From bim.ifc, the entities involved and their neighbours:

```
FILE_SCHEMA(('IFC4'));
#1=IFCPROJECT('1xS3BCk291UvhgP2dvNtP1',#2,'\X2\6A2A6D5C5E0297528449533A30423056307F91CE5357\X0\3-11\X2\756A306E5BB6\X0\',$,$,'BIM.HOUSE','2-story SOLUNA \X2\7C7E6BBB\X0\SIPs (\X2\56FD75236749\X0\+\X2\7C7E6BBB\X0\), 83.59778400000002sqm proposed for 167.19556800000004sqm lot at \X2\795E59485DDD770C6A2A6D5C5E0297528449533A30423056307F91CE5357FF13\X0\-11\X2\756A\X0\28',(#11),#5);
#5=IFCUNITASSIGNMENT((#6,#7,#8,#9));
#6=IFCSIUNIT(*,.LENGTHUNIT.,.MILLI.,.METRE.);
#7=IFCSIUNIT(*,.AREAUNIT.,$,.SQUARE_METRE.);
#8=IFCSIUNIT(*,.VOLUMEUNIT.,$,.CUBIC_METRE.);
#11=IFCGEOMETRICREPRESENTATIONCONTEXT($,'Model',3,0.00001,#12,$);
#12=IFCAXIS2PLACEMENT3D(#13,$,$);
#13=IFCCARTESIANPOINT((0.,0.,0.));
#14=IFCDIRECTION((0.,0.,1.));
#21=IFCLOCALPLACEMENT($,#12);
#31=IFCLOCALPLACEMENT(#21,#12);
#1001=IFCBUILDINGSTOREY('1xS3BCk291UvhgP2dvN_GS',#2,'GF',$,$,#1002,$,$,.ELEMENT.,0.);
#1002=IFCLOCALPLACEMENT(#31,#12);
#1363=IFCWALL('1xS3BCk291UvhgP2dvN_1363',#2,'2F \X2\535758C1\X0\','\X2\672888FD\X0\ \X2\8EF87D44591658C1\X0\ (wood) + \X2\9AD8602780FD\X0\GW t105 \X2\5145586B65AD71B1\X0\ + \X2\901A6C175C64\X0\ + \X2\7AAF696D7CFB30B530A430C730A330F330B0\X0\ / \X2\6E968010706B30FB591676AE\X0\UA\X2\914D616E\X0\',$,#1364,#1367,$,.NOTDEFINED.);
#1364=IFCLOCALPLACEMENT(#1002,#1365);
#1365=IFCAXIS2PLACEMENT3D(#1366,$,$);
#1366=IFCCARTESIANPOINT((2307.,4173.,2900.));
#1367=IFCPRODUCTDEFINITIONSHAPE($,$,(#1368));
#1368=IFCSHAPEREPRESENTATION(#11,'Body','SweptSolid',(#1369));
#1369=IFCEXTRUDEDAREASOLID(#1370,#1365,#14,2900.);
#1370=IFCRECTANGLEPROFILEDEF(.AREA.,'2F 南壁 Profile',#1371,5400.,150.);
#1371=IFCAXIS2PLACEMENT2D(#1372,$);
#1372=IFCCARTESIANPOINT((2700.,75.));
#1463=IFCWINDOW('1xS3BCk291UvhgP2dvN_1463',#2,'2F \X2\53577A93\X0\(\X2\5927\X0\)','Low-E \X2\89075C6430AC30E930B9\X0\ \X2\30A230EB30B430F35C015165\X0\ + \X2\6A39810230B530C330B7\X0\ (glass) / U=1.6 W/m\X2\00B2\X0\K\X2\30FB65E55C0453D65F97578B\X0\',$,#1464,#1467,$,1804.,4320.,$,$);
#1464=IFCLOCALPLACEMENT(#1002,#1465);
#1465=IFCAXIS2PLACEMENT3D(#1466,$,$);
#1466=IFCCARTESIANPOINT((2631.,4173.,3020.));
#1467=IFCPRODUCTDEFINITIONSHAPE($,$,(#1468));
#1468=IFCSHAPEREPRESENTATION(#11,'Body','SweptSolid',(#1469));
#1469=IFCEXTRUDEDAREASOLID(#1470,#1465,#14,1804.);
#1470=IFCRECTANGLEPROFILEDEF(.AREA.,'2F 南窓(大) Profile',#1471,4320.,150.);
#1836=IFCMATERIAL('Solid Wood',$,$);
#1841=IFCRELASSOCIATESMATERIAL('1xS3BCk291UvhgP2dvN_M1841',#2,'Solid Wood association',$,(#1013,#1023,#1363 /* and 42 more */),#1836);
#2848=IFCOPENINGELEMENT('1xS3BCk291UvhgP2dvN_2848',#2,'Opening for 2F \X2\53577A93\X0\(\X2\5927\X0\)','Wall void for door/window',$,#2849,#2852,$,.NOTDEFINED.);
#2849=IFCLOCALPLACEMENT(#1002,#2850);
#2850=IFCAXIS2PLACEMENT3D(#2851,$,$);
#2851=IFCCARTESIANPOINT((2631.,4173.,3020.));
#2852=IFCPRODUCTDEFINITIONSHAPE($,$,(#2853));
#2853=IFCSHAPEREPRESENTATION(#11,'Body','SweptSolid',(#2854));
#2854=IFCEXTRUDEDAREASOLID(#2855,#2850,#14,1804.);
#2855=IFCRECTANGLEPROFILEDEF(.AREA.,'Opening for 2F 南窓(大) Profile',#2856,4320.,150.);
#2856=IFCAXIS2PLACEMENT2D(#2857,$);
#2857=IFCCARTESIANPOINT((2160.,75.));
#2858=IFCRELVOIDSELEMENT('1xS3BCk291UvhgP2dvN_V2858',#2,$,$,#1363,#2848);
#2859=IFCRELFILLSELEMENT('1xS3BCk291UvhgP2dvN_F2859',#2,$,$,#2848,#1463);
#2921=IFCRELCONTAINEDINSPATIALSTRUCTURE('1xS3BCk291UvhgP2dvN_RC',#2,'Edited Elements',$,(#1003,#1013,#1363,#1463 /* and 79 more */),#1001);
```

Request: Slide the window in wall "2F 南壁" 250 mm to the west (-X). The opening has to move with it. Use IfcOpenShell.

```python
import ifcopenshell
import ifcopenshell.api.geometry
import ifcopenshell.util.placement
import ifcopenshell.util.unit

model = ifcopenshell.open("bim.ifc")
unit_scale = ifcopenshell.util.unit.calculate_unit_scale(model)

window = model.by_guid("1xS3BCk291UvhgP2dvN_1463")
opening = window.FillsVoids[0].RelatingOpeningElement
wall = opening.VoidsElements[0].RelatingBuildingElement

wall_matrix = ifcopenshell.util.placement.get_local_placement(wall.ObjectPlacement)
shift = wall_matrix[:3, 0] * -0.25 / unit_scale
before = ifcopenshell.util.placement.get_local_placement(window.ObjectPlacement)[:3, 3].copy()

# The window is not placed relative to its opening, so move both.
for product in (opening, window):
    matrix = ifcopenshell.util.placement.get_local_placement(product.ObjectPlacement)
    matrix[:3, 3] += shift
    ifcopenshell.api.geometry.edit_object_placement(model, product=product, matrix=matrix, is_si=False)

after = ifcopenshell.util.placement.get_local_placement(window.ObjectPlacement)[:3, 3]
print("window moved by", (after - before).round(3) + 0.0)

model.write("bim-out.ifc")
```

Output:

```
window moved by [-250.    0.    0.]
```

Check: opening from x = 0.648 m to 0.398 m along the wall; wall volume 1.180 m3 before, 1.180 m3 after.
